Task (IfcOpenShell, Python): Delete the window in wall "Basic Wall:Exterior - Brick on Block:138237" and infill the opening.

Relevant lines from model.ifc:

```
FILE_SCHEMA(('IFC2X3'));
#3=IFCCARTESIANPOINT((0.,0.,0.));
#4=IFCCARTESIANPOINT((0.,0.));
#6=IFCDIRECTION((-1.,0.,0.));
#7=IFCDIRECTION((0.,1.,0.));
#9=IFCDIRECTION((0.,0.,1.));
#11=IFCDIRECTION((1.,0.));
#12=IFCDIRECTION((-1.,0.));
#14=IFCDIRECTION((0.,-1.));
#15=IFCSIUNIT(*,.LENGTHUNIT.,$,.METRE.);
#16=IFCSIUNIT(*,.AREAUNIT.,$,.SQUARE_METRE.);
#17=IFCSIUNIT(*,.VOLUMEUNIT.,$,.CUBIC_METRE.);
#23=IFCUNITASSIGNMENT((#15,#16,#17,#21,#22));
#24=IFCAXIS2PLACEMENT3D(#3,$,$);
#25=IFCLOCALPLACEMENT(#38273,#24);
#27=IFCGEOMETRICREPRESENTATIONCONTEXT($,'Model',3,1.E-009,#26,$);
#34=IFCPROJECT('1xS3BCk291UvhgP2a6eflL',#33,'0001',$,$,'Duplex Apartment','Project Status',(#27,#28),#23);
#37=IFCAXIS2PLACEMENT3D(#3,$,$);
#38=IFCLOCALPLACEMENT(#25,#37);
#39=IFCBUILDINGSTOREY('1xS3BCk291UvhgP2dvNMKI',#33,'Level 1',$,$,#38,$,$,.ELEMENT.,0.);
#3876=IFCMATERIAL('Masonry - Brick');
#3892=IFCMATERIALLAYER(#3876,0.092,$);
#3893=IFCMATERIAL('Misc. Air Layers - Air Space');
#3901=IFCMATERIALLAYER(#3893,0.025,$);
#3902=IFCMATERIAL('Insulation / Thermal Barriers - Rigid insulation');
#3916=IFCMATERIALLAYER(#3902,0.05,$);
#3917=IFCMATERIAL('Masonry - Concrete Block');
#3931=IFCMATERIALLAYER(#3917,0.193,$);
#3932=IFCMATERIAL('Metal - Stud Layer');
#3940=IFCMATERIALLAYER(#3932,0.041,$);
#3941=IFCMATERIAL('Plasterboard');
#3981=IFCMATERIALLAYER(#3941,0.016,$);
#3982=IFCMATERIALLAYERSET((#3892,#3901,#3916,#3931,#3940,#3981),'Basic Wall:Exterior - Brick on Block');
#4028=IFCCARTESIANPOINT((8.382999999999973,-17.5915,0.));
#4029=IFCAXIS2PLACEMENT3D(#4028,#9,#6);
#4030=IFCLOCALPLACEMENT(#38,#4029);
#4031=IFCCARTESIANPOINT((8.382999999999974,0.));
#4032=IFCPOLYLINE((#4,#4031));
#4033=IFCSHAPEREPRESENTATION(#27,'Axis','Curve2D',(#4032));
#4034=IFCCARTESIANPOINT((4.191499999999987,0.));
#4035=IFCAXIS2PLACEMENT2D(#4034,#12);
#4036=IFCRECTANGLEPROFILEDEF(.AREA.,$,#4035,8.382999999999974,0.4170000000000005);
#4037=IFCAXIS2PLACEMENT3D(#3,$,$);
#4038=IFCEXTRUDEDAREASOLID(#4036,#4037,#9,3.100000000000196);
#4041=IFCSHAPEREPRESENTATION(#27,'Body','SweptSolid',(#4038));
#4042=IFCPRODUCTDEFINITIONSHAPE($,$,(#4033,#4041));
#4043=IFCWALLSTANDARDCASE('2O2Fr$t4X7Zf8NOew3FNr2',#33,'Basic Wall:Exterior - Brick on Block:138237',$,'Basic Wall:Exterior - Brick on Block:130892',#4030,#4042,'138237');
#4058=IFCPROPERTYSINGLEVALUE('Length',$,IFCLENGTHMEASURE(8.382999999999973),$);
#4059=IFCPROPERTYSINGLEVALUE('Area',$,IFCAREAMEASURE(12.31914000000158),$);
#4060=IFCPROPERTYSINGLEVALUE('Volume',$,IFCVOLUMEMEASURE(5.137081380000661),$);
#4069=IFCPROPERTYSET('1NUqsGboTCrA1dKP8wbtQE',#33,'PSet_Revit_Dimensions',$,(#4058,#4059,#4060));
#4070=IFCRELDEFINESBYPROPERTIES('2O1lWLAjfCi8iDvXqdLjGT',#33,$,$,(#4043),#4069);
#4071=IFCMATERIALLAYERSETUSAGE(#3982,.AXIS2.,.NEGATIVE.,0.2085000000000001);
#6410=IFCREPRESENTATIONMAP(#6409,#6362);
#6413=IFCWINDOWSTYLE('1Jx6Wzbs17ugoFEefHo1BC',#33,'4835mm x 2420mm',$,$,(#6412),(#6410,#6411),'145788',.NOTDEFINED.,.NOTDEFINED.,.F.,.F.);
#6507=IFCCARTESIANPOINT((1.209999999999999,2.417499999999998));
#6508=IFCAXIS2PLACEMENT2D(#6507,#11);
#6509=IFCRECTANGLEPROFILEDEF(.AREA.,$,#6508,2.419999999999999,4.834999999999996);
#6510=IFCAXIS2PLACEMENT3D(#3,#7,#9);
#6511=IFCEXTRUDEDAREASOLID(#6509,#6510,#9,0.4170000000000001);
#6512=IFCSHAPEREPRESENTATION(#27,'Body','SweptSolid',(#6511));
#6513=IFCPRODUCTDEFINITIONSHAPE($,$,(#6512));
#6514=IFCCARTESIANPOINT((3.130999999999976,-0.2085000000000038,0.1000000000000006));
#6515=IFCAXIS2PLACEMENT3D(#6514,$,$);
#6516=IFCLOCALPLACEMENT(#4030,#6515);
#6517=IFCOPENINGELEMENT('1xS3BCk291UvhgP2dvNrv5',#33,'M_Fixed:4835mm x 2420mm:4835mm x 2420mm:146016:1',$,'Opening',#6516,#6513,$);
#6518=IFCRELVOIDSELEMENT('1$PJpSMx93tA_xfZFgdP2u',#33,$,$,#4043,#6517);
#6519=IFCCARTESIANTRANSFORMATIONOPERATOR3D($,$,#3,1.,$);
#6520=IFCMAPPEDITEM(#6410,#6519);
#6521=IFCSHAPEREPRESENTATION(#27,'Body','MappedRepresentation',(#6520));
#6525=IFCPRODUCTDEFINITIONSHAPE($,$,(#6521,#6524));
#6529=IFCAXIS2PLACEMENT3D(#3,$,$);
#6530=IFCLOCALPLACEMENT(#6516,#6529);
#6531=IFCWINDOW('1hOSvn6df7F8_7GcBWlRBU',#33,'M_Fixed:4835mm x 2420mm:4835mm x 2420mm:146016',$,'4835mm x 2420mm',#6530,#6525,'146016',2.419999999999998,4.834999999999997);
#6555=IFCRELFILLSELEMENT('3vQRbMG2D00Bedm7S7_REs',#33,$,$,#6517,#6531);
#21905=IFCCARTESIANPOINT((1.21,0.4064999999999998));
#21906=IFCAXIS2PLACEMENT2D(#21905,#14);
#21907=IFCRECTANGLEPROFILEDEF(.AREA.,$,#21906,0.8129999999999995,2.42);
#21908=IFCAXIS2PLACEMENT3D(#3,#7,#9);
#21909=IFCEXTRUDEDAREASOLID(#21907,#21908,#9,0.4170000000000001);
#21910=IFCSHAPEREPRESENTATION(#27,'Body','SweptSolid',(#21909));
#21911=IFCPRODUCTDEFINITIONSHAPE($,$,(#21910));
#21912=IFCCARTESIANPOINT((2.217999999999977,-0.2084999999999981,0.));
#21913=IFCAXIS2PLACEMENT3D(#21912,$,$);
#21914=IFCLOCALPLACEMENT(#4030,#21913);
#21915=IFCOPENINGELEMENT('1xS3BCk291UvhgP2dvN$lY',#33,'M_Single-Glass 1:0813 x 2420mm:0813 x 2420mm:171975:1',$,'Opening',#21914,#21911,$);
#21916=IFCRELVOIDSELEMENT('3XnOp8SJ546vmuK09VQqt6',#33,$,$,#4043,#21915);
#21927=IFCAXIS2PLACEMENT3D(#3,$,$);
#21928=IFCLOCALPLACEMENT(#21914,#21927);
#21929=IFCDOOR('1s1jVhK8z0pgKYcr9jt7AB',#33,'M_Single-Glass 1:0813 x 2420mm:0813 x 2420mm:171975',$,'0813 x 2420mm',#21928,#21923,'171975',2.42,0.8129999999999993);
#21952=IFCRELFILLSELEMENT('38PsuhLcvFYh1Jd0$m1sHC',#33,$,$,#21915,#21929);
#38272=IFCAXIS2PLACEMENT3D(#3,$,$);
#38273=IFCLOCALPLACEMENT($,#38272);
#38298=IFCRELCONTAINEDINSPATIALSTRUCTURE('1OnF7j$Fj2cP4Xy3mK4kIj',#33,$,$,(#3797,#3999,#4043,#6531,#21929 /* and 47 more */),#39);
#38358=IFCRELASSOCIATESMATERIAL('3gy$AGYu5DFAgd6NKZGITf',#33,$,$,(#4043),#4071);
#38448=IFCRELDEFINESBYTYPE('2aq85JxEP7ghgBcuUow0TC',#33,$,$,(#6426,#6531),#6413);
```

```python
import ifcopenshell
import ifcopenshell.api.feature
import ifcopenshell.api.pset
import ifcopenshell.api.root
import ifcopenshell.geom
import ifcopenshell.util.element
import ifcopenshell.util.shape
import ifcopenshell.util.unit

model = ifcopenshell.open("model.ifc")
area_scale = ifcopenshell.util.unit.calculate_unit_scale(model, "AREAUNIT")
volume_scale = ifcopenshell.util.unit.calculate_unit_scale(model, "VOLUMEUNIT")
settings = ifcopenshell.geom.settings()


def volume(element):
    """Net volume in cubic metres, openings subtracted."""
    shape = ifcopenshell.geom.create_shape(settings, element)
    return ifcopenshell.util.shape.get_volume(shape.geometry)


window = model.by_id(6531)
opening = window.FillsVoids[0].RelatingOpeningElement
wall = opening.VoidsElements[0].RelatingBuildingElement
before = volume(wall)

ifcopenshell.api.root.remove_product(model, product=window)
ifcopenshell.api.feature.remove_feature(model, feature=opening)

after = volume(wall)
thickness = 0.417  # wall thickness in metres

# Update the wall's stored quantities.
pset = model.by_id(ifcopenshell.util.element.get_pset(wall, "PSet_Revit_Dimensions", should_inherit=False)["id"])
ifcopenshell.api.pset.edit_pset(model, pset=pset, properties={
    "Area": model.create_entity("IfcAreaMeasure", after / thickness / area_scale),
    "Volume": model.create_entity("IfcVolumeMeasure", after / volume_scale),
})

print(f"wall volume {before:.3f} -> {after:.3f} m3")

model.write("model_v2.ifc")
```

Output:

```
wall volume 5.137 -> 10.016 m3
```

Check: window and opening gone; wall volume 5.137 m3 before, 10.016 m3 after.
